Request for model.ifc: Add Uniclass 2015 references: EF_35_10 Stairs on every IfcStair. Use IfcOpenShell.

First a look at what the model holds.

```python
import ifcopenshell

model = ifcopenshell.open("model.ifc")
print(model.schema)
print("classifications:", [c.Name for c in model.by_type("IfcClassification")])
for ifc_class in ("IfcDoor", "IfcRoof", "IfcStair", "IfcWall", "IfcWindow"):
    print(ifc_class, len(model.by_type(ifc_class)))
```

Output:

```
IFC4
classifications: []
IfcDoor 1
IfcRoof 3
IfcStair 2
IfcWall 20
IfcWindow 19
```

```python
import ifcopenshell
import ifcopenshell.api.classification

model = ifcopenshell.open("model.ifc")

system = ifcopenshell.api.classification.add_classification(model, classification="Uniclass 2015")

codes = {
    "IfcStair": ("EF_35_10", "Stairs"),
}
for ifc_class, (code, name) in codes.items():
    products = model.by_type(ifc_class)
    ifcopenshell.api.classification.add_reference(
        model, products=products, classification=system, identification=code, name=name
    )
    print(code, len(products))

model.write("model_v2.ifc")
```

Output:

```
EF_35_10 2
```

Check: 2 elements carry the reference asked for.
